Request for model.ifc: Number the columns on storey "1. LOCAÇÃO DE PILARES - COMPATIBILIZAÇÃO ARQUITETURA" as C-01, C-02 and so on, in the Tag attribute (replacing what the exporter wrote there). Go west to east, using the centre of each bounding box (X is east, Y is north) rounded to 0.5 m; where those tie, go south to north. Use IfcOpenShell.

First a look at what the model holds.

```python
import ifcopenshell
import ifcopenshell.util.element
import ifcopenshell.util.placement

model = ifcopenshell.open("model.ifc")
print(model.schema)
storey = next(s for s in model.by_type("IfcBuildingStorey") if s.Name == "1. LOCAÇÃO DE PILARES - COMPATIBILIZAÇÃO ARQUITETURA")
columns = [e for e in ifcopenshell.util.element.get_decomposition(storey) if e.is_a("IfcColumn")]
for e in sorted(columns, key=lambda e: e.id()):
    origin = ifcopenshell.util.placement.get_local_placement(e.ObjectPlacement)[:3, 3]
    print(e.id(), e.Tag, e.Name, origin.round(2) + 0.0, sep=" | ")
```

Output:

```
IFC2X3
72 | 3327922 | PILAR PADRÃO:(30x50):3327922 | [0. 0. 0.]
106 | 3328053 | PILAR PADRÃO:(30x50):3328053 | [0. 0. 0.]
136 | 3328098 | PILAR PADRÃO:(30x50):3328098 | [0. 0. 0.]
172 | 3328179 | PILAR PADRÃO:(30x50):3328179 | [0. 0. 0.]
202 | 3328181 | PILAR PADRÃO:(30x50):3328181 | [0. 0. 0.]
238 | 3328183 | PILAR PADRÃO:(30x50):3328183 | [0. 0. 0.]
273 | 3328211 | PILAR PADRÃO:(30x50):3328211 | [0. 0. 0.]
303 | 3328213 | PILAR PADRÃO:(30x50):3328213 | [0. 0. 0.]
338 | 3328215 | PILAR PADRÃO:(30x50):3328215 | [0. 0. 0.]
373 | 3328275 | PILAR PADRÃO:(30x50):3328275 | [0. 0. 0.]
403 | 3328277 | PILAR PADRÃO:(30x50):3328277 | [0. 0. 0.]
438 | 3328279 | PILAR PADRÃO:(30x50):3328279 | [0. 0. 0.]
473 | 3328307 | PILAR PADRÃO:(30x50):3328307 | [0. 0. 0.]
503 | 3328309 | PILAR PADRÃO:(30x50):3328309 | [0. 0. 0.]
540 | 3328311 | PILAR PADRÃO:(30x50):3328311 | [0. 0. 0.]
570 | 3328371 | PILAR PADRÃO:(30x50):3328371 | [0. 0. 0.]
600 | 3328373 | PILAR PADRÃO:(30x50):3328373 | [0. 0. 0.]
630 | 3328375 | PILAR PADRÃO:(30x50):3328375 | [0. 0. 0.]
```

```python
import ifcopenshell
import ifcopenshell.geom
import ifcopenshell.util.element
import ifcopenshell.util.shape

model = ifcopenshell.open("model.ifc")
settings = ifcopenshell.geom.settings()
settings.set("use-world-coords", True)


def centre(element):
    shape = ifcopenshell.geom.create_shape(settings, element)
    return ifcopenshell.util.shape.get_bbox_centroid(shape.geometry)


storey = next(s for s in model.by_type("IfcBuildingStorey") if s.Name == "1. LOCAÇÃO DE PILARES - COMPATIBILIZAÇÃO ARQUITETURA")
columns = [e for e in ifcopenshell.util.element.get_decomposition(storey) if e.is_a("IfcColumn")]

# Insertion points can sit at a corner or the storey origin, so sort by the geometry (in metres).
centres = {e: centre(e) for e in columns}
columns.sort(key=lambda e: (round(centres[e][0] / 0.5), centres[e][1]))

for i, e in enumerate(columns, start=1):
    number = f"C-{i:02d}"
    e.Tag = number
    print(e.id(), number)

model.write("model_rev.ifc")
```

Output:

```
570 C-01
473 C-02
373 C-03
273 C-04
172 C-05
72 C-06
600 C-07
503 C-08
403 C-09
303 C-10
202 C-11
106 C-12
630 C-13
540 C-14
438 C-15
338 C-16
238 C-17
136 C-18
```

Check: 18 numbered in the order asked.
